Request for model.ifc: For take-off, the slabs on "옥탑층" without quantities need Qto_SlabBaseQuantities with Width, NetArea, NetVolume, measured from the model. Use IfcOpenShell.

First a look at what the model holds.

```python
import ifcopenshell
import ifcopenshell.util.element
import ifcopenshell.util.unit

model = ifcopenshell.open("model.ifc")
print(model.schema)
for unit_type in ("LENGTHUNIT", "AREAUNIT", "VOLUMEUNIT"):
    print(unit_type, ifcopenshell.util.unit.calculate_unit_scale(model, unit_type))
storey = next(s for s in model.by_type("IfcBuildingStorey") if s.Name == "옥탑층")
slabs = [e for e in ifcopenshell.util.element.get_decomposition(storey) if e.is_a("IfcSlab")]
for e in sorted(slabs, key=lambda e: e.id()):
    print(e.id(), e.is_a(), e.Name, list(ifcopenshell.util.element.get_psets(e, qtos_only=True)), sep=" | ")
```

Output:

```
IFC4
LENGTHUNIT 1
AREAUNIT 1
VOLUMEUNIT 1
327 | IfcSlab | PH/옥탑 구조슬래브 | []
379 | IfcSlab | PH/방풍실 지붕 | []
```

```python
import ifcopenshell
import ifcopenshell.api.pset
import ifcopenshell.geom
import ifcopenshell.util.element
import ifcopenshell.util.shape
import ifcopenshell.util.unit

model = ifcopenshell.open("model.ifc")
unit_scale = ifcopenshell.util.unit.calculate_unit_scale(model)
area_scale = ifcopenshell.util.unit.calculate_unit_scale(model, "AREAUNIT")
volume_scale = ifcopenshell.util.unit.calculate_unit_scale(model, "VOLUMEUNIT")
settings = ifcopenshell.geom.settings()

storey = next(s for s in model.by_type("IfcBuildingStorey") if s.Name == "옥탑층")
slabs = [e for e in ifcopenshell.util.element.get_decomposition(storey) if e.is_a("IfcSlab")]

for e in sorted(slabs, key=lambda e: e.id()):
    if ifcopenshell.util.element.get_psets(e, qtos_only=True, should_inherit=False):
        continue
    # Geometry comes back in metres, in the element's own axes.
    shape = ifcopenshell.geom.create_shape(settings, e)
    values = {
        "Width": ifcopenshell.util.shape.get_z(shape.geometry) / unit_scale,
        "NetArea": ifcopenshell.util.shape.get_footprint_area(shape.geometry) / area_scale,
        "NetVolume": ifcopenshell.util.shape.get_volume(shape.geometry) / volume_scale,
    }
    qto = ifcopenshell.api.pset.add_qto(model, product=e, name="Qto_SlabBaseQuantities")
    ifcopenshell.api.pset.edit_qto(model, qto=qto, properties=values)
    print(e.id(), {k: round(v, 3) for k, v in values.items()})

model.write("model-out.ifc")
```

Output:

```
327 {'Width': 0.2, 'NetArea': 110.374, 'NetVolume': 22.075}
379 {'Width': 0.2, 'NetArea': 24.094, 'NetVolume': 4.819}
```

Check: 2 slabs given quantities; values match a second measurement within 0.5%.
